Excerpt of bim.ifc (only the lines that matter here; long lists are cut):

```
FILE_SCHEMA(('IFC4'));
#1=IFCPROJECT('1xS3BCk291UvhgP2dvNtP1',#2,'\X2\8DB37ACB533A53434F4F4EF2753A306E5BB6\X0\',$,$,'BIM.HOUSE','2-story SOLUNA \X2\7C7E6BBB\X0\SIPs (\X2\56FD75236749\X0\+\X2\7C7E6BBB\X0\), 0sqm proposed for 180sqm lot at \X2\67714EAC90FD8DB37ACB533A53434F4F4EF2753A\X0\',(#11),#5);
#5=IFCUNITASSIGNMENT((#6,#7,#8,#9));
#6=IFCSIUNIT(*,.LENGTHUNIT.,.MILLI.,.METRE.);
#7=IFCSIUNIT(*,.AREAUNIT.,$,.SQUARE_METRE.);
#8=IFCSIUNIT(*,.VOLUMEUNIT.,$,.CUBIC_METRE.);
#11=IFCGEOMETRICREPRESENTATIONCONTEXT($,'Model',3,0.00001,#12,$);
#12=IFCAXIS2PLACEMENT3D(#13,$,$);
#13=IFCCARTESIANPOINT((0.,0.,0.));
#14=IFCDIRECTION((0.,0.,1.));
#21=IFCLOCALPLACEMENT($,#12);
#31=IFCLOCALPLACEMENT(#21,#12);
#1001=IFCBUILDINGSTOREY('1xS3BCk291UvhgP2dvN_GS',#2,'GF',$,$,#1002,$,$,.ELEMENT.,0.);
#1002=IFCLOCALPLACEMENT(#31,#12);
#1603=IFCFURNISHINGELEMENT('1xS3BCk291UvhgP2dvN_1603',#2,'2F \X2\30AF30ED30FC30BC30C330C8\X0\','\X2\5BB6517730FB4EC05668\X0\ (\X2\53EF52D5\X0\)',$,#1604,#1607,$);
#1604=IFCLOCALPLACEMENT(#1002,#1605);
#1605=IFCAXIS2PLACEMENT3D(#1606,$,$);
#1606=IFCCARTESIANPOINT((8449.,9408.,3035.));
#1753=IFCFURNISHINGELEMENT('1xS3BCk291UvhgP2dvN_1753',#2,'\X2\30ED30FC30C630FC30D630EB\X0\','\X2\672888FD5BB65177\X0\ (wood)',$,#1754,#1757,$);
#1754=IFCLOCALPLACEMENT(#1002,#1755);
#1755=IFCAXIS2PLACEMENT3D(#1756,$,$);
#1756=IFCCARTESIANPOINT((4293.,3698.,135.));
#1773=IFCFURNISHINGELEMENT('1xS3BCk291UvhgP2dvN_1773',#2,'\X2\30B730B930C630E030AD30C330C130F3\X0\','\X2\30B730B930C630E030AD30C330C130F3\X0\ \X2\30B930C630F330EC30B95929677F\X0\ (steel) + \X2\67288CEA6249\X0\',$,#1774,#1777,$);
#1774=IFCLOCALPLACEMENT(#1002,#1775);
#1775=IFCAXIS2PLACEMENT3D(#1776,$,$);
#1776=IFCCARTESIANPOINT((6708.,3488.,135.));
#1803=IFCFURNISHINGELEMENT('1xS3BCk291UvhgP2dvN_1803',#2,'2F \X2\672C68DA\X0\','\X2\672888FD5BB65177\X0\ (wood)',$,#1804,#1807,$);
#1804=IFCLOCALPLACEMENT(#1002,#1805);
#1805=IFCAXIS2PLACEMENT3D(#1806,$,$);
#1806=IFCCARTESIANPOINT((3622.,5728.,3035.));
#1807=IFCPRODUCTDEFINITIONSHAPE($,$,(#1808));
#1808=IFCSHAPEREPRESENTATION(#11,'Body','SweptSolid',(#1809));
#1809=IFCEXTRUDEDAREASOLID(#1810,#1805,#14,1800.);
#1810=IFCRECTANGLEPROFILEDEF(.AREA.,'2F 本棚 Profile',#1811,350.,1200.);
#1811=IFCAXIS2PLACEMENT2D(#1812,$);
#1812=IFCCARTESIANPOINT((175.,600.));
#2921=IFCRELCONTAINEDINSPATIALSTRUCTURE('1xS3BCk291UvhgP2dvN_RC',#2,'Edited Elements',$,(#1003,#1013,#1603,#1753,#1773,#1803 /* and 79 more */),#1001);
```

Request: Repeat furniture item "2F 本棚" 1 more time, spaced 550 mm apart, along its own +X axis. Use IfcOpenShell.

```python
import ifcopenshell
import ifcopenshell.api.geometry
import ifcopenshell.api.root
import ifcopenshell.util.element
import ifcopenshell.util.placement
import ifcopenshell.util.unit

model = ifcopenshell.open("bim.ifc")
unit_scale = ifcopenshell.util.unit.calculate_unit_scale(model)


def reuse_history(source, copy):
    """copy_class also copies each property set's owner history, people and application; keep the originals."""
    for rel in copy.IsDefinedBy:
        if rel.is_a("IfcRelDefinesByProperties") and (history := rel.RelatingPropertyDefinition.OwnerHistory):
            rel.RelatingPropertyDefinition.OwnerHistory = source.OwnerHistory
            ifcopenshell.util.element.remove_deep2(model, history)


source = model.by_guid("1xS3BCk291UvhgP2dvN_1803")
base = ifcopenshell.util.placement.get_local_placement(source.ObjectPlacement)
step = base[:3, 0] * 0.55 / unit_scale

for i in range(1, 2):
    copy = ifcopenshell.api.root.copy_class(model, product=source)
    copy.Representation = ifcopenshell.util.element.copy_deep(
        model, source.Representation, exclude=["IfcGeometricRepresentationContext", "IfcRepresentationMap"]
    )
    reuse_history(source, copy)
    matrix = base.copy()
    matrix[:3, 3] += i * step
    print("added at", matrix[:3, 3].round(3) + 0.0)
    ifcopenshell.api.geometry.edit_object_placement(model, product=copy, matrix=matrix, is_si=False)

model.write("bim_v2.ifc")
```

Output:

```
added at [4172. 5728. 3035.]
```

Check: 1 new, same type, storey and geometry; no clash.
